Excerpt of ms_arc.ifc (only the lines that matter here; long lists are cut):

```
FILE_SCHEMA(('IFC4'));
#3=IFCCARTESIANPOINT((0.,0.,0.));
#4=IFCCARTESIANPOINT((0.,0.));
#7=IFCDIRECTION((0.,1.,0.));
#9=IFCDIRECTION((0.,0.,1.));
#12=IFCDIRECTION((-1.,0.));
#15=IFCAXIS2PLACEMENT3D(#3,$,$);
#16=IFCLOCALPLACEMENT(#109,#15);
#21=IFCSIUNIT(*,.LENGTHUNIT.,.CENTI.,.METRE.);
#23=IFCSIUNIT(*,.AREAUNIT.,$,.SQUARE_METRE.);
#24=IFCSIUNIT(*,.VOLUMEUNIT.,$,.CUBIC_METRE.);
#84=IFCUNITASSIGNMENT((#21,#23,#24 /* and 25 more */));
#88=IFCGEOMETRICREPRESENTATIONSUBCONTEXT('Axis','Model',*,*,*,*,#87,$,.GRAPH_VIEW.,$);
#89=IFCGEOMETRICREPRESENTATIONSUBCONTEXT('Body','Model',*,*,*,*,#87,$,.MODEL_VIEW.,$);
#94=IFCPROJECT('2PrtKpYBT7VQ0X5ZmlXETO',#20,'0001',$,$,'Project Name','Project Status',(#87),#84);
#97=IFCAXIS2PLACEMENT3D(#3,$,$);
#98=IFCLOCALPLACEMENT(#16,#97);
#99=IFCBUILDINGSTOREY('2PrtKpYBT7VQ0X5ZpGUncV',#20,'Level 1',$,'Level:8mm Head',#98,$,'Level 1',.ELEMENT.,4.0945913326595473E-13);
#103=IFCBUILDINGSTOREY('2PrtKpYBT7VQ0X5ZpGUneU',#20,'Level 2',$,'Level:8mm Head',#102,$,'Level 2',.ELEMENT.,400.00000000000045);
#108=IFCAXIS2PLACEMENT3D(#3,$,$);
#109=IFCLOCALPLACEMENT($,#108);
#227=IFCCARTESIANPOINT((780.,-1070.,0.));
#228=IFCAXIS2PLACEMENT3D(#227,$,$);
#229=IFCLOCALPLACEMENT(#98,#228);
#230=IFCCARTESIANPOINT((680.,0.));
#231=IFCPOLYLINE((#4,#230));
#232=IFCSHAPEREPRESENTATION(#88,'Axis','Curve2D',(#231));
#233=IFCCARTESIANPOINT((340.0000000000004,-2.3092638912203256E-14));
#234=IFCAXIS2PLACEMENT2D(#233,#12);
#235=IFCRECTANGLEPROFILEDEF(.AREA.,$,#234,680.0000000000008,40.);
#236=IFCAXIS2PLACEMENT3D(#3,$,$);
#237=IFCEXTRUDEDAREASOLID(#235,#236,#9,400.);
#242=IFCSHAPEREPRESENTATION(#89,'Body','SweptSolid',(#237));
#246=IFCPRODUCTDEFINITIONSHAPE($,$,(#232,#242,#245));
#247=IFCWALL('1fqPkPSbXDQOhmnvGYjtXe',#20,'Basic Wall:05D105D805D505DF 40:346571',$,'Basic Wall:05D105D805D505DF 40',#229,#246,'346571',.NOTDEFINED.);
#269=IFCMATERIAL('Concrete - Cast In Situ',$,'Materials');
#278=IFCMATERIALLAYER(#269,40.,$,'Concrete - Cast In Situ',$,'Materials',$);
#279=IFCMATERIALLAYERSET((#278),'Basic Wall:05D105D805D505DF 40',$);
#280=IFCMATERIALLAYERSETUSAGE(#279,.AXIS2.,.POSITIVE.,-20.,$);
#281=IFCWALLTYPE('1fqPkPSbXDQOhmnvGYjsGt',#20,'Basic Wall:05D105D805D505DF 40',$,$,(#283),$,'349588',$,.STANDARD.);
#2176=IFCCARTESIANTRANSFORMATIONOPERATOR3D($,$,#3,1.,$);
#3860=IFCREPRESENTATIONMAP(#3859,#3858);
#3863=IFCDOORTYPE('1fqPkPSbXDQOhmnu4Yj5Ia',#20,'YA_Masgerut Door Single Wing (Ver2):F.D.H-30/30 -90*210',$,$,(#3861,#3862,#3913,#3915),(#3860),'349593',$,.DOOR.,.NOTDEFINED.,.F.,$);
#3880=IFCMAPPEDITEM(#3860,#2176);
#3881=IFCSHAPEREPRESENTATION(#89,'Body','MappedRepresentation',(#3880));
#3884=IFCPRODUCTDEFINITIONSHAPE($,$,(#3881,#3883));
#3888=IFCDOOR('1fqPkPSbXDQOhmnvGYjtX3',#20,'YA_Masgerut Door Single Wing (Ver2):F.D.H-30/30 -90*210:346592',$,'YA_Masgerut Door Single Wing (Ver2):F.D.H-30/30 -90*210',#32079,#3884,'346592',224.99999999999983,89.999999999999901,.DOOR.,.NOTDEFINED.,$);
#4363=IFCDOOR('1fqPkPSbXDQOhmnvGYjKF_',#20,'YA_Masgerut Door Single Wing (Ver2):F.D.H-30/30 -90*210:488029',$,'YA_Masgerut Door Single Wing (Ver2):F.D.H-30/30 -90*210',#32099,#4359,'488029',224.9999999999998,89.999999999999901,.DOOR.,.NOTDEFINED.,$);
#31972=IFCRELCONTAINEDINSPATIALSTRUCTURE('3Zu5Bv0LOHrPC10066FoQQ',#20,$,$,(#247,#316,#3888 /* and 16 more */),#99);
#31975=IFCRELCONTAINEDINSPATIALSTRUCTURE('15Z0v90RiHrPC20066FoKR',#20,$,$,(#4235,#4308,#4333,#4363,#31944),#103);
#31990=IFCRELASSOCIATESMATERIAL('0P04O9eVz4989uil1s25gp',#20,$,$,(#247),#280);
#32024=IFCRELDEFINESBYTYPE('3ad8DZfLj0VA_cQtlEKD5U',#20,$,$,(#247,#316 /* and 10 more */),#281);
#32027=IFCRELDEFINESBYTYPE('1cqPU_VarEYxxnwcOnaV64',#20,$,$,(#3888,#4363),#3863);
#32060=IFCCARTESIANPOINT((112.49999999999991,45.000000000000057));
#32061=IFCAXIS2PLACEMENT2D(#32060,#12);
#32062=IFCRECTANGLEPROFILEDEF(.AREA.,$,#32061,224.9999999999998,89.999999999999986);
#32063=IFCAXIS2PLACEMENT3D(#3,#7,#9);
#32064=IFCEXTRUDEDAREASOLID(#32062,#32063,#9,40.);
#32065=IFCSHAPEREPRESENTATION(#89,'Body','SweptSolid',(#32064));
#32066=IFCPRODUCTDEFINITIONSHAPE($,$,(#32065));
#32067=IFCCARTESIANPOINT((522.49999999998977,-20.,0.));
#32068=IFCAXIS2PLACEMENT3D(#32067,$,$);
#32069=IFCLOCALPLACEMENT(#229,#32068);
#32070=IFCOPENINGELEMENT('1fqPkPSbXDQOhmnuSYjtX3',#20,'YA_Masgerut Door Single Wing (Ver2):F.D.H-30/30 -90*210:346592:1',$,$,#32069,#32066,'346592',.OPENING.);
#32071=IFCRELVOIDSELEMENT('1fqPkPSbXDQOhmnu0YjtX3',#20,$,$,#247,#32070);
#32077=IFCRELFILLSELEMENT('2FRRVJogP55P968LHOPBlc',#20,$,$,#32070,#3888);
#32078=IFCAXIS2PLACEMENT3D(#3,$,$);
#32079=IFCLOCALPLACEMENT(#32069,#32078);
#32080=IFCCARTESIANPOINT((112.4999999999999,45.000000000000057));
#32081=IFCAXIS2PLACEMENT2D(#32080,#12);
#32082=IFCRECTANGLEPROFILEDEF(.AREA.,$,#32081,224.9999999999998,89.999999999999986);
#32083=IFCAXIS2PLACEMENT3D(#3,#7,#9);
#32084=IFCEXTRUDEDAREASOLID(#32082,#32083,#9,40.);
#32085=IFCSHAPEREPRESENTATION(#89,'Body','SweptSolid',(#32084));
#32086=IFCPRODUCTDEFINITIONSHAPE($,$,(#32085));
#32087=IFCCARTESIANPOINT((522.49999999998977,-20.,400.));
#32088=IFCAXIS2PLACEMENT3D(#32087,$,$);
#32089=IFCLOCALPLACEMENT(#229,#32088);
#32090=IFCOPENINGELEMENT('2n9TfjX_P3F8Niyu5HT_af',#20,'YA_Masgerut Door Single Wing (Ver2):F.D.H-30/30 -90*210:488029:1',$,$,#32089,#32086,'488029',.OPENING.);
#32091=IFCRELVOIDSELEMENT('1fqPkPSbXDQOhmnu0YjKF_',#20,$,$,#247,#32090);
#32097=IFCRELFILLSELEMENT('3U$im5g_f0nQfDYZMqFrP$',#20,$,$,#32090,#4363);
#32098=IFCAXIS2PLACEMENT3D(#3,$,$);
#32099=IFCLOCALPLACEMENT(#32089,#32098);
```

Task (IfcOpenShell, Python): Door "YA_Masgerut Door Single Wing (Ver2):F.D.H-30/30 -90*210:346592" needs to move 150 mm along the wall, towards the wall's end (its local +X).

```python
import ifcopenshell
import ifcopenshell.api.geometry
import ifcopenshell.util.placement
import ifcopenshell.util.unit

model = ifcopenshell.open("ms_arc.ifc")
unit_scale = ifcopenshell.util.unit.calculate_unit_scale(model)

door = model.by_id(3888)
opening = door.FillsVoids[0].RelatingOpeningElement
wall = opening.VoidsElements[0].RelatingBuildingElement

wall_matrix = ifcopenshell.util.placement.get_local_placement(wall.ObjectPlacement)
shift = wall_matrix[:3, 0] * 0.15 / unit_scale
before = ifcopenshell.util.placement.get_local_placement(door.ObjectPlacement)[:3, 3].copy()

# The door is placed relative to its opening, so it follows when the opening moves.
matrix = ifcopenshell.util.placement.get_local_placement(opening.ObjectPlacement)
matrix[:3, 3] += shift
ifcopenshell.api.geometry.edit_object_placement(
    model, product=opening, matrix=matrix, is_si=False, should_transform_children=True
)

after = ifcopenshell.util.placement.get_local_placement(door.ObjectPlacement)[:3, 3]
print("door moved by", (after - before).round(3) + 0.0)

model.write("ms_arc_rev.ifc")
```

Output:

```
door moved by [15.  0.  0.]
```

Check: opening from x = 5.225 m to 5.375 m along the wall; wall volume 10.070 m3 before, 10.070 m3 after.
